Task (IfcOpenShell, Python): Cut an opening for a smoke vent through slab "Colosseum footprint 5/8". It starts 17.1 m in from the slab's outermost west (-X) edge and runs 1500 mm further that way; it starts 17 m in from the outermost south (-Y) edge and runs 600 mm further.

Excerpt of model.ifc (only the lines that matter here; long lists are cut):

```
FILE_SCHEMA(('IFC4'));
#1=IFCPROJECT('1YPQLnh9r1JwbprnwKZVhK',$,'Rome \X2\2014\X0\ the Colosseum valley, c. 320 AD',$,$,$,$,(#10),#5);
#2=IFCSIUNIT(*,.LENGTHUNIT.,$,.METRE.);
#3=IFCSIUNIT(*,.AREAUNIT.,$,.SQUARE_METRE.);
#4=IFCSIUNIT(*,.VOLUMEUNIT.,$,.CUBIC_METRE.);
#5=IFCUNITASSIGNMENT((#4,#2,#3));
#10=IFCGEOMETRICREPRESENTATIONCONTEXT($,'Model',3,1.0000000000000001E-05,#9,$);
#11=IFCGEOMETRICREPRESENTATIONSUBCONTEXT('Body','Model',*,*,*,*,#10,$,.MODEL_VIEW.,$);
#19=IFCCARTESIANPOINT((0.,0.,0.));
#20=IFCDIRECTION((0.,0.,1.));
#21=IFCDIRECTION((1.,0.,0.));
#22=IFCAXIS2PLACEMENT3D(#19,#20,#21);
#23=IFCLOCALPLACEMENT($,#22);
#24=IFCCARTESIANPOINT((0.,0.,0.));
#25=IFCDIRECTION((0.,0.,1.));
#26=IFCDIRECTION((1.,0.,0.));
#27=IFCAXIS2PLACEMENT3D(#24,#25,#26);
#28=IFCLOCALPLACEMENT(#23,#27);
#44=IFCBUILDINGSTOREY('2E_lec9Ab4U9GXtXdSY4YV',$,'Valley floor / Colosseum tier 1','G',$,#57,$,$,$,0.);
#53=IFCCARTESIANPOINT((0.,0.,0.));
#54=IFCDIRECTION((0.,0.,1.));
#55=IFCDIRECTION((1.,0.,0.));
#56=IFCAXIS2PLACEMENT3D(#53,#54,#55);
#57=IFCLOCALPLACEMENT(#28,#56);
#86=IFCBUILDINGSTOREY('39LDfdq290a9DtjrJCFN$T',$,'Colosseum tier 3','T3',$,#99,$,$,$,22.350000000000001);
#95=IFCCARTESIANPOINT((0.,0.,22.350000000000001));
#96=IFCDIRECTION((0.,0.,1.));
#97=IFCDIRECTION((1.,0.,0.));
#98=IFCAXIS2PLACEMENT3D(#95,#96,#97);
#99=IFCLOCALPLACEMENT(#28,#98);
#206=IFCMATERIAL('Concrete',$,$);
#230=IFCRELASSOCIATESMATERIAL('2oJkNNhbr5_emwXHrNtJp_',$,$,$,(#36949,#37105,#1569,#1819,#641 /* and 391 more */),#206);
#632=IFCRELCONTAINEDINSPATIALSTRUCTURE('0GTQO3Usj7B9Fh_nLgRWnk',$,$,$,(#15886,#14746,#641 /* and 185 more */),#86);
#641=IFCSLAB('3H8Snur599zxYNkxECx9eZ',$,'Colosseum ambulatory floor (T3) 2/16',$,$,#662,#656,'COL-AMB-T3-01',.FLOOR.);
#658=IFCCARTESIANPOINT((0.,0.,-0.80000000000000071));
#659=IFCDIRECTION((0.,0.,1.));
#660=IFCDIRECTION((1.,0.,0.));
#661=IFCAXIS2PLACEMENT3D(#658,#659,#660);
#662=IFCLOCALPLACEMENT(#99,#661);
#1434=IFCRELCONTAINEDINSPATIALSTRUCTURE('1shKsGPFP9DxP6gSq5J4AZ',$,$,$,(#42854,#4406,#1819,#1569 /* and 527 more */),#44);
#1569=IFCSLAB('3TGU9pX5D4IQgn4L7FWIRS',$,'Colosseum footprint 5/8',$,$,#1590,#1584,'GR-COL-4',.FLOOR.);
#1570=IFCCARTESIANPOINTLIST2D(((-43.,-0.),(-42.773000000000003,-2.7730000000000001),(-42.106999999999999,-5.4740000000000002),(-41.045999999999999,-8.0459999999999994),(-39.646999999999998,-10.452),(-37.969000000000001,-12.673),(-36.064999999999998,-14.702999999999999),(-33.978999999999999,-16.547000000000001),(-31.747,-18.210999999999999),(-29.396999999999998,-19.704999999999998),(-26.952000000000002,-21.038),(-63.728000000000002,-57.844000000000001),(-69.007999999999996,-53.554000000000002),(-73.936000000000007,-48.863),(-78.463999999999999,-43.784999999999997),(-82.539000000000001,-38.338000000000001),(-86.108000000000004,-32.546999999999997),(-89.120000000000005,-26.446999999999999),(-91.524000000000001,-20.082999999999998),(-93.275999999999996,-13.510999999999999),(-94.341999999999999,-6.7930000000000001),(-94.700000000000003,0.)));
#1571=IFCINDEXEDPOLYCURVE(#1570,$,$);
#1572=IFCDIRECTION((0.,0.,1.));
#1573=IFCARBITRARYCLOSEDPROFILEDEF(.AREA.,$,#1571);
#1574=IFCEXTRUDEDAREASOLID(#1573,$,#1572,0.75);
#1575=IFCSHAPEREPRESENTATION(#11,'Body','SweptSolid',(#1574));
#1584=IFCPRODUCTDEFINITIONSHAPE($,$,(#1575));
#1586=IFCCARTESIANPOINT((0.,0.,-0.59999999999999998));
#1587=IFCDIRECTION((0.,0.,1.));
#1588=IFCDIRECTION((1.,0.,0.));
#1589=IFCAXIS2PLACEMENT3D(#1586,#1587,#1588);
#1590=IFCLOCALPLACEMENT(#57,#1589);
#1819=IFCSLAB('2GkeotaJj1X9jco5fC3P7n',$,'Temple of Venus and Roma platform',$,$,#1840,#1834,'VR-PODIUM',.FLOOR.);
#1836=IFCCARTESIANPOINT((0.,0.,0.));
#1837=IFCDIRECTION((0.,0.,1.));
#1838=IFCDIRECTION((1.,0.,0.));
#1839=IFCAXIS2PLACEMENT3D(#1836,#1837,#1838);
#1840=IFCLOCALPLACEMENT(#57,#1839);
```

```python
import numpy as np
import ifcopenshell
import ifcopenshell.api.feature
import ifcopenshell.api.geometry
import ifcopenshell.api.root
import ifcopenshell.geom
import ifcopenshell.util.placement
import ifcopenshell.util.representation
import ifcopenshell.util.shape
import ifcopenshell.util.unit

model = ifcopenshell.open("model.ifc")
unit_scale = ifcopenshell.util.unit.calculate_unit_scale(model)
settings = ifcopenshell.geom.settings()


def volume(element):
    """Net volume in cubic metres, openings subtracted."""
    shape = ifcopenshell.geom.create_shape(settings, element)
    return ifcopenshell.util.shape.get_volume(shape.geometry)


slab = model.by_guid("3TGU9pX5D4IQgn4L7FWIRS")
before = volume(slab)

# Extent in the slab's own axes, in metres. The edges named are its -X and -Y sides.
slab_shape = ifcopenshell.geom.create_shape(settings, slab)
vertices = ifcopenshell.util.shape.get_vertices(slab_shape.geometry)
x_min, y_min, bottom = vertices.min(axis=0)
top = vertices[:, 2].max()

opening = ifcopenshell.api.root.create_entity(model, ifc_class="IfcOpeningElement", name="Smoke vent opening", predefined_type="OPENING")
context = ifcopenshell.util.representation.get_context(model, "Model", "Body", "MODEL_VIEW")
width, depth = 1.5, 0.6
outline = [(0.0, 0.0), (width, 0.0), (width, depth), (0.0, depth), (0.0, 0.0)]
# Overshoot both faces by 50 mm so the cut is clean.
shape = ifcopenshell.api.geometry.add_slab_representation(
    model, context=context, depth=top - bottom + 0.1, polyline=outline
)
ifcopenshell.api.geometry.assign_representation(model, product=opening, representation=shape)

matrix = ifcopenshell.util.placement.get_local_placement(slab.ObjectPlacement)
matrix[:, 3] = matrix @ np.append(np.array([x_min + 17.1, y_min + 17, bottom - 0.05]) / unit_scale, 1.0)
ifcopenshell.api.geometry.edit_object_placement(model, product=opening, matrix=matrix, is_si=False)
ifcopenshell.api.feature.add_feature(model, feature=opening, element=slab)

after = volume(slab)

print(f"slab volume {before:.3f} -> {after:.3f} m3")

model.write("model_edited.ifc")
```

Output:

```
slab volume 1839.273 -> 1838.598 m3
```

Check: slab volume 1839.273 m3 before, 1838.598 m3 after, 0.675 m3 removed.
